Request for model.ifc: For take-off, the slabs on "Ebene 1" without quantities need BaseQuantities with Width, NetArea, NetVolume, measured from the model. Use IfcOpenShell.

First a look at what the model holds.

```python
import ifcopenshell
import ifcopenshell.util.element
import ifcopenshell.util.unit

model = ifcopenshell.open("model.ifc")
print(model.schema)
for unit_type in ("LENGTHUNIT", "AREAUNIT", "VOLUMEUNIT"):
    print(unit_type, ifcopenshell.util.unit.calculate_unit_scale(model, unit_type))
storey = next(s for s in model.by_type("IfcBuildingStorey") if s.Name == "Ebene 1")
slabs = [e for e in ifcopenshell.util.element.get_decomposition(storey) if e.is_a("IfcSlab")]
for e in sorted(slabs, key=lambda e: e.id()):
    print(e.id(), e.is_a(), e.Name, list(ifcopenshell.util.element.get_psets(e, qtos_only=True)), sep=" | ")
```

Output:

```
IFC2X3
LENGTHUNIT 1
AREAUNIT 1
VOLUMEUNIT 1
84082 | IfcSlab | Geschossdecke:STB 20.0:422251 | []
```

```python
import ifcopenshell
import ifcopenshell.api.pset
import ifcopenshell.geom
import ifcopenshell.util.element
import ifcopenshell.util.shape
import ifcopenshell.util.unit

model = ifcopenshell.open("model.ifc")
unit_scale = ifcopenshell.util.unit.calculate_unit_scale(model)
area_scale = ifcopenshell.util.unit.calculate_unit_scale(model, "AREAUNIT")
volume_scale = ifcopenshell.util.unit.calculate_unit_scale(model, "VOLUMEUNIT")
settings = ifcopenshell.geom.settings()

storey = next(s for s in model.by_type("IfcBuildingStorey") if s.Name == "Ebene 1")
slabs = [e for e in ifcopenshell.util.element.get_decomposition(storey) if e.is_a("IfcSlab")]

for e in sorted(slabs, key=lambda e: e.id()):
    if ifcopenshell.util.element.get_psets(e, qtos_only=True, should_inherit=False):
        continue
    # Geometry comes back in metres, in the element's own axes.
    shape = ifcopenshell.geom.create_shape(settings, e)
    values = {
        "Width": ifcopenshell.util.shape.get_z(shape.geometry) / unit_scale,
        "NetArea": ifcopenshell.util.shape.get_footprint_area(shape.geometry) / area_scale,
        "NetVolume": ifcopenshell.util.shape.get_volume(shape.geometry) / volume_scale,
    }
    qto = ifcopenshell.api.pset.add_qto(model, product=e, name="BaseQuantities")
    ifcopenshell.api.pset.edit_qto(model, qto=qto, properties=values)
    print(e.id(), {k: round(v, 3) for k, v in values.items()})

model.write("model_rev.ifc")
```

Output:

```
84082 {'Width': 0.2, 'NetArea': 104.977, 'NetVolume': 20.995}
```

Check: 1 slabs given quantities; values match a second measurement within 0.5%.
